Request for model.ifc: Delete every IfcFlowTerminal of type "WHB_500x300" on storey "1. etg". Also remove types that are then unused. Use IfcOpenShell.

First a look at what the model holds.

```python
import ifcopenshell
import ifcopenshell.util.element

model = ifcopenshell.open("model.ifc")
print(model.schema)
storey = next(s for s in model.by_type("IfcBuildingStorey") if s.Name == "1. etg")
terminals = [e for e in ifcopenshell.util.element.get_decomposition(storey) if e.is_a("IfcFlowTerminal")]
seen = {}
for e in terminals:
    element_type = ifcopenshell.util.element.get_type(e)
    name = element_type.Name if element_type not in (None, e) else None
    seen[name] = seen.get(name, 0) + 1
for name, count in sorted(seen.items(), key=str):
    print(count, "x", name)
```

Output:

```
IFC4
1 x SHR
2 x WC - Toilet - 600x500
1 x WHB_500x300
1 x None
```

```python
import ifcopenshell
import ifcopenshell.api.root
import ifcopenshell.util.element

model = ifcopenshell.open("model.ifc")

storey = next(s for s in model.by_type("IfcBuildingStorey") if s.Name == "1. etg")
terminals = [e for e in ifcopenshell.util.element.get_decomposition(storey) if e.is_a("IfcFlowTerminal")]
targets = [e for e in terminals if (t := ifcopenshell.util.element.get_type(e)) not in (None, e) and t.Name == "WHB_500x300"]
types = {ifcopenshell.util.element.get_type(e) for e in targets} - {None, *targets}

for e in targets:
    ifcopenshell.api.root.remove_product(model, product=e)
print(len(targets), "removed")

unused = [t for t in types if not ifcopenshell.util.element.get_types(t)]
for t in unused:
    ifcopenshell.api.root.remove_product(model, product=t)
print(len(unused), "unused types removed")

model.write("model-out.ifc")
```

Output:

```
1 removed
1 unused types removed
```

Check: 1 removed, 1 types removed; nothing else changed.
